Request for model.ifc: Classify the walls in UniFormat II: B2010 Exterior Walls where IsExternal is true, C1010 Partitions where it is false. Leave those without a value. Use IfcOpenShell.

First a look at what the model holds.

```python
import ifcopenshell
import ifcopenshell.util.element

model = ifcopenshell.open("model.ifc")
print(model.schema)
print("classifications:", [c.Name for c in model.by_type("IfcClassification")])
values = [ifcopenshell.util.element.get_pset(e, "Pset_WallCommon", "IsExternal") for e in model.by_type("IfcWall")]
for value in (True, False, None):
    print("IsExternal", value, values.count(value))
```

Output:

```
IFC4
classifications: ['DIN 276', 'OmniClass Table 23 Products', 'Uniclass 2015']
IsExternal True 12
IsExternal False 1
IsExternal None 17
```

```python
import ifcopenshell
import ifcopenshell.api.classification
import ifcopenshell.util.element

model = ifcopenshell.open("model.ifc")

system = ifcopenshell.api.classification.add_classification(model, classification="UniFormat II")

walls = model.by_type("IfcWall")
external = {e: ifcopenshell.util.element.get_pset(e, "Pset_WallCommon", "IsExternal") for e in walls}
for flag, code, name in ((True, "B2010", "Exterior Walls"), (False, "C1010", "Partitions")):
    products = [e for e in walls if external[e] is flag]
    ifcopenshell.api.classification.add_reference(
        model, products=products, classification=system, identification=code, name=name
    )
    print(code, len(products))

model.write("model_edited.ifc")
```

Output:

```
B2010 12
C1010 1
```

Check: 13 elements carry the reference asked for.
